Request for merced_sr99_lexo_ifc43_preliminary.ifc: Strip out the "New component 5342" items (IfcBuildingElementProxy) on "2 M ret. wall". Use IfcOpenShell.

First a look at what the model holds.

```python
import ifcopenshell
import ifcopenshell.util.element

model = ifcopenshell.open("merced_sr99_lexo_ifc43_preliminary.ifc")
print(model.schema)
storey = next(s for s in model.by_type("IfcBuildingStorey") if s.Name == "2 M ret. wall")
proxies = [e for e in ifcopenshell.util.element.get_decomposition(storey) if e.is_a("IfcBuildingElementProxy")]
seen = {}
for e in proxies:
    element_type = ifcopenshell.util.element.get_type(e)
    name = element_type.Name if element_type not in (None, e) else None
    seen[name] = seen.get(name, 0) + 1
for name, count in sorted(seen.items(), key=str):
    print(count, "x", name)
```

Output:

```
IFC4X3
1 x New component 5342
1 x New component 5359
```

```python
import ifcopenshell
import ifcopenshell.api.root
import ifcopenshell.util.element

model = ifcopenshell.open("merced_sr99_lexo_ifc43_preliminary.ifc")

storey = next(s for s in model.by_type("IfcBuildingStorey") if s.Name == "2 M ret. wall")
proxies = [e for e in ifcopenshell.util.element.get_decomposition(storey) if e.is_a("IfcBuildingElementProxy")]
targets = [e for e in proxies if (t := ifcopenshell.util.element.get_type(e)) not in (None, e) and t.Name == "New component 5342"]

for e in targets:
    ifcopenshell.api.root.remove_product(model, product=e)
print(len(targets), "removed")

model.write("merced_sr99_lexo_ifc43_preliminary-out.ifc")
```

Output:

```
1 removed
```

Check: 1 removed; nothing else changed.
